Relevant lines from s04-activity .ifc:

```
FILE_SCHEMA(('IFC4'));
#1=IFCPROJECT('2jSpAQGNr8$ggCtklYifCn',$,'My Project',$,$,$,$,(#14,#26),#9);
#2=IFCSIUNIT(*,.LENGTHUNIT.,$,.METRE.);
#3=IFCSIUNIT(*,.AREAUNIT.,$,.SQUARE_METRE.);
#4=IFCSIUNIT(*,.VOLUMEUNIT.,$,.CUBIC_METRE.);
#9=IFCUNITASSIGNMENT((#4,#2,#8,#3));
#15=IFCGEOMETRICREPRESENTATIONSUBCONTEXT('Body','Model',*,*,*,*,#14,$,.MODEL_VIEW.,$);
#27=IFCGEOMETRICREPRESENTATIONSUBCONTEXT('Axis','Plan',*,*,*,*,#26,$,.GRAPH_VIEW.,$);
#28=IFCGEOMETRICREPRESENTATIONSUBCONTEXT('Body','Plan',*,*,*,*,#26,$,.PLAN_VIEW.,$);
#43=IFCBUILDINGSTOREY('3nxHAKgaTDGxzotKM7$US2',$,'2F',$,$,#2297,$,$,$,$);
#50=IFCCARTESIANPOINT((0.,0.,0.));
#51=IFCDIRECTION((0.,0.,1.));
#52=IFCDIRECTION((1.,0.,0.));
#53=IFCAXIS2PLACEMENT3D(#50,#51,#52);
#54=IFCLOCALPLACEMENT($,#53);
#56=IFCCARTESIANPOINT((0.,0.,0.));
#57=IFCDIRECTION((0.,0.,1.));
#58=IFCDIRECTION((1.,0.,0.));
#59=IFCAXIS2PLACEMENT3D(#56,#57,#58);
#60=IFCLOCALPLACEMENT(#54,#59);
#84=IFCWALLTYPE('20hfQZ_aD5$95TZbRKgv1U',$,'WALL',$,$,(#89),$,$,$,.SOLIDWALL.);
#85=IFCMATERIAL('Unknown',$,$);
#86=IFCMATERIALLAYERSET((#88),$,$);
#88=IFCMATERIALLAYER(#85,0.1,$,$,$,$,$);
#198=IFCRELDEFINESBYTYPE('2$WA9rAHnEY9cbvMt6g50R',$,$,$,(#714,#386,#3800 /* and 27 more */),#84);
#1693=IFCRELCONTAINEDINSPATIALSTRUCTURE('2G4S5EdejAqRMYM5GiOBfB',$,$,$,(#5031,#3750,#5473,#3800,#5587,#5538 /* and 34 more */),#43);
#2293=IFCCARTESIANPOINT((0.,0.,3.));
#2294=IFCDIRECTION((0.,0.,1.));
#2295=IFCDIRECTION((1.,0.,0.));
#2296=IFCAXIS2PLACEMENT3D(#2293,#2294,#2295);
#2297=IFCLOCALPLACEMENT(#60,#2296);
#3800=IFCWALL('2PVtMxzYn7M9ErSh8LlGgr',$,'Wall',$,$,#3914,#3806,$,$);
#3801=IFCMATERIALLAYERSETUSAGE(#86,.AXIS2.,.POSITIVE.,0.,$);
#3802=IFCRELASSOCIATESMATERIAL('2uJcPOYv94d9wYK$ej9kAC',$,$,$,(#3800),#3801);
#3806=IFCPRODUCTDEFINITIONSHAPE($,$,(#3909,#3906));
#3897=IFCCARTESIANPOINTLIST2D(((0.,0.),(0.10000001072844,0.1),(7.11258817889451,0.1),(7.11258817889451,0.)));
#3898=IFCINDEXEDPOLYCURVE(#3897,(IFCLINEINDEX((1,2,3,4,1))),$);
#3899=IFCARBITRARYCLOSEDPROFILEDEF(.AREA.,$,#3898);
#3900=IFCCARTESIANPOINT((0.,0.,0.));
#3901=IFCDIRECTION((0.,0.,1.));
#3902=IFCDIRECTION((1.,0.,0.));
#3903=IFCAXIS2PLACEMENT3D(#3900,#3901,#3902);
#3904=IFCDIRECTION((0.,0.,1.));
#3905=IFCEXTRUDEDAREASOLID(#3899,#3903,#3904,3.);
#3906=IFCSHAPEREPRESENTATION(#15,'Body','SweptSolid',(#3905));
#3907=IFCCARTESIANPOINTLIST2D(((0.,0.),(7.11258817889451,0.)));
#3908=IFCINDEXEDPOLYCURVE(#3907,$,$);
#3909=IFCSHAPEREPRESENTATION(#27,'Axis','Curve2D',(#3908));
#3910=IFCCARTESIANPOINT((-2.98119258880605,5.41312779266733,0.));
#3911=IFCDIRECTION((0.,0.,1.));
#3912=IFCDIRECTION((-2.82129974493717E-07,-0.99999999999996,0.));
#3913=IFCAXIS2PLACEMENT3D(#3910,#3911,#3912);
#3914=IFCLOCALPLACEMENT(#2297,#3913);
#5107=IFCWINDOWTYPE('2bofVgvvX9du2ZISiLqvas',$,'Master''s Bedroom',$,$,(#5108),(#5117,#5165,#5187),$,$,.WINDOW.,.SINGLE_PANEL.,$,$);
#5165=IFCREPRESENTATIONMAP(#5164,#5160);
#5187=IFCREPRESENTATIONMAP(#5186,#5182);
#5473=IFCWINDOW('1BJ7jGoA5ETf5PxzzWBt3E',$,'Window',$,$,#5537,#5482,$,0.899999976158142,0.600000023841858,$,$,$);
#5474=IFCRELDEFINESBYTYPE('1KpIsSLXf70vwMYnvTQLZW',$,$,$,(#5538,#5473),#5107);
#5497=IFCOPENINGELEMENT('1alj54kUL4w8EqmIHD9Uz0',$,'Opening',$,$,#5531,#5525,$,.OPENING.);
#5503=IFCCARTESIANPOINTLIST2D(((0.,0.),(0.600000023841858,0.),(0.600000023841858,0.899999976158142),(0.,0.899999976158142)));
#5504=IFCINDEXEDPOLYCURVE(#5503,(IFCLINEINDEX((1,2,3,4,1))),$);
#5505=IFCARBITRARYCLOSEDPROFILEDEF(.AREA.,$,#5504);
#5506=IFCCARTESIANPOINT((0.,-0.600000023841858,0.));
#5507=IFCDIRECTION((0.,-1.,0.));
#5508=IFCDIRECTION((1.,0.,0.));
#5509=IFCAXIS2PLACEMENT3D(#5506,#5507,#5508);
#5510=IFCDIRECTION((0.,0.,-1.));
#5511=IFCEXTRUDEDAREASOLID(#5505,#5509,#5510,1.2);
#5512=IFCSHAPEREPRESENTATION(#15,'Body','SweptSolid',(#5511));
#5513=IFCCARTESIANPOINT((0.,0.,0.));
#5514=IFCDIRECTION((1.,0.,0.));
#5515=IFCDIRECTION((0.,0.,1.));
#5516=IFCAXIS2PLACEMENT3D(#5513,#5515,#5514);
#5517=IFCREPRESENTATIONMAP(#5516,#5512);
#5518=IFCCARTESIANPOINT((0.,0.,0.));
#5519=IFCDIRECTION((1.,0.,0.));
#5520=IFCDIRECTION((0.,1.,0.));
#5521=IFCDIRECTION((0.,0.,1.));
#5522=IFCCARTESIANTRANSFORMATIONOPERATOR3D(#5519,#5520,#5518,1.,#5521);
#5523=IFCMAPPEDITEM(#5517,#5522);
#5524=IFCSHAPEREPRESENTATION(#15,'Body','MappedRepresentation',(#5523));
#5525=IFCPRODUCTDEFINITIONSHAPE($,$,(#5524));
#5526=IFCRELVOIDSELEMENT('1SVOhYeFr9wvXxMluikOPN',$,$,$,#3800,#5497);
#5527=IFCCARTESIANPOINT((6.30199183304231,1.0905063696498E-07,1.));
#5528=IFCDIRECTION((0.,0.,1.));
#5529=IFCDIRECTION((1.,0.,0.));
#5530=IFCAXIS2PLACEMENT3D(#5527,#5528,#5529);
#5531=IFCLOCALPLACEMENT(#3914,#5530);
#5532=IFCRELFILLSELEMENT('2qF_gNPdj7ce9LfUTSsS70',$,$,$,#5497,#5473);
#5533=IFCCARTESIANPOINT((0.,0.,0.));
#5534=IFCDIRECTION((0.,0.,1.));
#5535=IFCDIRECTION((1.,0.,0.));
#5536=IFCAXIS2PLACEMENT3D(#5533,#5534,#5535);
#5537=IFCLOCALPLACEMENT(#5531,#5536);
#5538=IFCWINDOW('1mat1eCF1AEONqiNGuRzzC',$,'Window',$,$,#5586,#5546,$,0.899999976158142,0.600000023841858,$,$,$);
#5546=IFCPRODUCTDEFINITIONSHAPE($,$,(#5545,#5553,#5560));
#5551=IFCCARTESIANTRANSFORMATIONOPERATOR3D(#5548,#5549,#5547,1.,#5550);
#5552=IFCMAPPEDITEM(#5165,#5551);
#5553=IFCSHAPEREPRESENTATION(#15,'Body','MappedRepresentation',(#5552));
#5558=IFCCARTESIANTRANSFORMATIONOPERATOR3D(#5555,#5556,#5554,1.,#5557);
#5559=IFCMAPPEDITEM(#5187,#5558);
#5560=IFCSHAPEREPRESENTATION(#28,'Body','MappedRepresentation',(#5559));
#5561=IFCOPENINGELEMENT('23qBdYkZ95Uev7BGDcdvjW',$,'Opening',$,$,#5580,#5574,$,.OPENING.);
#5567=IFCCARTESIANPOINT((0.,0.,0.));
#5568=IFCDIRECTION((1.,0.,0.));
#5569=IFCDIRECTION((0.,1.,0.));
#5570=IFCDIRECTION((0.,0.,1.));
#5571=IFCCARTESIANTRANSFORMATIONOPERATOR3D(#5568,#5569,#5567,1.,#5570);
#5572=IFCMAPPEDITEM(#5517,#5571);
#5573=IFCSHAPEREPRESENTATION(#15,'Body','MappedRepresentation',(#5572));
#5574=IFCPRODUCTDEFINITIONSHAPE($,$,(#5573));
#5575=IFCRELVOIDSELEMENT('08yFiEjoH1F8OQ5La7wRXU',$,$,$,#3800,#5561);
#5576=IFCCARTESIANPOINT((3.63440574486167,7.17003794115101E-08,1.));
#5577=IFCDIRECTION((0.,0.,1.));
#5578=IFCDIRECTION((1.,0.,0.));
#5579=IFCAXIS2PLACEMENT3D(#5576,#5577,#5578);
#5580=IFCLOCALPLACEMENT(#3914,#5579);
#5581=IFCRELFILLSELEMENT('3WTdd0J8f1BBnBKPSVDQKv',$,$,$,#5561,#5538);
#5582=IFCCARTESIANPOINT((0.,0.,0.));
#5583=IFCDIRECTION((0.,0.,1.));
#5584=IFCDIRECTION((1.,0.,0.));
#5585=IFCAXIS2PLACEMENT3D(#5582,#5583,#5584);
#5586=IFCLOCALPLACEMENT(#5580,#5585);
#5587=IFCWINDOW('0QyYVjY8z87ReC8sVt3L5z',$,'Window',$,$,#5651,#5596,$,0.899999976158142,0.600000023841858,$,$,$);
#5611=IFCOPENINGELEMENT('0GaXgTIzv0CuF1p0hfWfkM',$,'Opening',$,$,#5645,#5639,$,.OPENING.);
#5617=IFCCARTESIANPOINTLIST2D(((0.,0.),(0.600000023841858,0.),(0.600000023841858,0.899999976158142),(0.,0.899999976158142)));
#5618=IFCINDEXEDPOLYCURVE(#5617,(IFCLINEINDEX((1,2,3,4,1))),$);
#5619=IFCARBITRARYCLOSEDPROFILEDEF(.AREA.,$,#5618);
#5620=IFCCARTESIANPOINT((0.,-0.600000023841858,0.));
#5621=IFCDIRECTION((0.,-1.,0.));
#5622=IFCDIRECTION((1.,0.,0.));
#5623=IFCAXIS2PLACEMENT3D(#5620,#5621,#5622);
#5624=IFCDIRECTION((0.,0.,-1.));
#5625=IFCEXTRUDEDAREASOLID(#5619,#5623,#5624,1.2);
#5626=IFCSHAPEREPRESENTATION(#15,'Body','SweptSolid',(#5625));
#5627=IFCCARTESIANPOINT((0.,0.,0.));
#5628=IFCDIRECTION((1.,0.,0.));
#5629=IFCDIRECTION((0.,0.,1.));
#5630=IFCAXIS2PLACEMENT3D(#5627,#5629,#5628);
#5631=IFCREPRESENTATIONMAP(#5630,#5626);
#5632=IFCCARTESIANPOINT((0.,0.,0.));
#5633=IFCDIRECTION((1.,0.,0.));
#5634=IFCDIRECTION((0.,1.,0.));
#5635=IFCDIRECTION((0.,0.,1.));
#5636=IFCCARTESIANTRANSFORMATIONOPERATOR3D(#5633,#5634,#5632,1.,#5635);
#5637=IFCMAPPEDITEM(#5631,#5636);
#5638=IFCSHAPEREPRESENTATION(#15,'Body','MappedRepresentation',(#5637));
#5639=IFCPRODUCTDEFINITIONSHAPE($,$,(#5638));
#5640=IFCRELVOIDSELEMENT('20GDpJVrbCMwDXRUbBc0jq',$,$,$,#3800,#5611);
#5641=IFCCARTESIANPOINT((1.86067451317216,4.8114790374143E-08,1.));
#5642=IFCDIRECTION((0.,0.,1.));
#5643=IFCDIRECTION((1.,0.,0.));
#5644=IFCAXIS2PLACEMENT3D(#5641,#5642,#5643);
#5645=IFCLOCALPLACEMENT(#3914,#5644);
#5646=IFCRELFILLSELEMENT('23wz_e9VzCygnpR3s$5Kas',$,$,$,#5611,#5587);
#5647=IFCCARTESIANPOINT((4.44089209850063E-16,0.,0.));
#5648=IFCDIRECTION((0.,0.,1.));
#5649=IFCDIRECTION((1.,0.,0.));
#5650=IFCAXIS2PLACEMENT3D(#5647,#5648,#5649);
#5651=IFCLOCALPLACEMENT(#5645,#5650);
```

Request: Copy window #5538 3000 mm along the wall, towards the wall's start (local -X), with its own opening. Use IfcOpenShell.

```python
import ifcopenshell
import ifcopenshell.api.feature
import ifcopenshell.api.geometry
import ifcopenshell.api.root
import ifcopenshell.geom
import ifcopenshell.util.element
import ifcopenshell.util.placement
import ifcopenshell.util.shape
import ifcopenshell.util.unit

model = ifcopenshell.open("s04-activity .ifc")
unit_scale = ifcopenshell.util.unit.calculate_unit_scale(model)
settings = ifcopenshell.geom.settings()


def volume(element):
    """Net volume in cubic metres, openings subtracted."""
    shape = ifcopenshell.geom.create_shape(settings, element)
    return ifcopenshell.util.shape.get_volume(shape.geometry)


window = model.by_guid("1mat1eCF1AEONqiNGuRzzC")
opening = window.FillsVoids[0].RelatingOpeningElement
wall = opening.VoidsElements[0].RelatingBuildingElement
before = volume(wall)
shift = ifcopenshell.util.placement.get_local_placement(wall.ObjectPlacement)[:3, 0] * -3 / unit_scale

# copy_class copies the void relationship, type, container and properties, but no geometry.
new_opening = ifcopenshell.api.root.copy_class(model, product=opening)
new_opening.Representation = ifcopenshell.util.element.copy_deep(
    model, opening.Representation, exclude=["IfcGeometricRepresentationContext", "IfcRepresentationMap"]
)
new_window = ifcopenshell.api.root.copy_class(model, product=window)
new_window.Representation = ifcopenshell.util.element.copy_deep(
    model, window.Representation, exclude=["IfcGeometricRepresentationContext", "IfcRepresentationMap"]
)
ifcopenshell.api.feature.add_filling(model, opening=new_opening, element=new_window)

for old, new in ((opening, new_opening), (window, new_window)):
    matrix = ifcopenshell.util.placement.get_local_placement(old.ObjectPlacement)
    matrix[:3, 3] += shift
    ifcopenshell.api.geometry.edit_object_placement(model, product=new, matrix=matrix, is_si=False)

after = volume(wall)

print(f"wall volume {before:.3f} -> {after:.3f} m3")

model.write("s04-activity _v2.ifc")
```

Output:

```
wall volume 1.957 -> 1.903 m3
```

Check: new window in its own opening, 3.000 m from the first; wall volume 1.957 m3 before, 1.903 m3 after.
